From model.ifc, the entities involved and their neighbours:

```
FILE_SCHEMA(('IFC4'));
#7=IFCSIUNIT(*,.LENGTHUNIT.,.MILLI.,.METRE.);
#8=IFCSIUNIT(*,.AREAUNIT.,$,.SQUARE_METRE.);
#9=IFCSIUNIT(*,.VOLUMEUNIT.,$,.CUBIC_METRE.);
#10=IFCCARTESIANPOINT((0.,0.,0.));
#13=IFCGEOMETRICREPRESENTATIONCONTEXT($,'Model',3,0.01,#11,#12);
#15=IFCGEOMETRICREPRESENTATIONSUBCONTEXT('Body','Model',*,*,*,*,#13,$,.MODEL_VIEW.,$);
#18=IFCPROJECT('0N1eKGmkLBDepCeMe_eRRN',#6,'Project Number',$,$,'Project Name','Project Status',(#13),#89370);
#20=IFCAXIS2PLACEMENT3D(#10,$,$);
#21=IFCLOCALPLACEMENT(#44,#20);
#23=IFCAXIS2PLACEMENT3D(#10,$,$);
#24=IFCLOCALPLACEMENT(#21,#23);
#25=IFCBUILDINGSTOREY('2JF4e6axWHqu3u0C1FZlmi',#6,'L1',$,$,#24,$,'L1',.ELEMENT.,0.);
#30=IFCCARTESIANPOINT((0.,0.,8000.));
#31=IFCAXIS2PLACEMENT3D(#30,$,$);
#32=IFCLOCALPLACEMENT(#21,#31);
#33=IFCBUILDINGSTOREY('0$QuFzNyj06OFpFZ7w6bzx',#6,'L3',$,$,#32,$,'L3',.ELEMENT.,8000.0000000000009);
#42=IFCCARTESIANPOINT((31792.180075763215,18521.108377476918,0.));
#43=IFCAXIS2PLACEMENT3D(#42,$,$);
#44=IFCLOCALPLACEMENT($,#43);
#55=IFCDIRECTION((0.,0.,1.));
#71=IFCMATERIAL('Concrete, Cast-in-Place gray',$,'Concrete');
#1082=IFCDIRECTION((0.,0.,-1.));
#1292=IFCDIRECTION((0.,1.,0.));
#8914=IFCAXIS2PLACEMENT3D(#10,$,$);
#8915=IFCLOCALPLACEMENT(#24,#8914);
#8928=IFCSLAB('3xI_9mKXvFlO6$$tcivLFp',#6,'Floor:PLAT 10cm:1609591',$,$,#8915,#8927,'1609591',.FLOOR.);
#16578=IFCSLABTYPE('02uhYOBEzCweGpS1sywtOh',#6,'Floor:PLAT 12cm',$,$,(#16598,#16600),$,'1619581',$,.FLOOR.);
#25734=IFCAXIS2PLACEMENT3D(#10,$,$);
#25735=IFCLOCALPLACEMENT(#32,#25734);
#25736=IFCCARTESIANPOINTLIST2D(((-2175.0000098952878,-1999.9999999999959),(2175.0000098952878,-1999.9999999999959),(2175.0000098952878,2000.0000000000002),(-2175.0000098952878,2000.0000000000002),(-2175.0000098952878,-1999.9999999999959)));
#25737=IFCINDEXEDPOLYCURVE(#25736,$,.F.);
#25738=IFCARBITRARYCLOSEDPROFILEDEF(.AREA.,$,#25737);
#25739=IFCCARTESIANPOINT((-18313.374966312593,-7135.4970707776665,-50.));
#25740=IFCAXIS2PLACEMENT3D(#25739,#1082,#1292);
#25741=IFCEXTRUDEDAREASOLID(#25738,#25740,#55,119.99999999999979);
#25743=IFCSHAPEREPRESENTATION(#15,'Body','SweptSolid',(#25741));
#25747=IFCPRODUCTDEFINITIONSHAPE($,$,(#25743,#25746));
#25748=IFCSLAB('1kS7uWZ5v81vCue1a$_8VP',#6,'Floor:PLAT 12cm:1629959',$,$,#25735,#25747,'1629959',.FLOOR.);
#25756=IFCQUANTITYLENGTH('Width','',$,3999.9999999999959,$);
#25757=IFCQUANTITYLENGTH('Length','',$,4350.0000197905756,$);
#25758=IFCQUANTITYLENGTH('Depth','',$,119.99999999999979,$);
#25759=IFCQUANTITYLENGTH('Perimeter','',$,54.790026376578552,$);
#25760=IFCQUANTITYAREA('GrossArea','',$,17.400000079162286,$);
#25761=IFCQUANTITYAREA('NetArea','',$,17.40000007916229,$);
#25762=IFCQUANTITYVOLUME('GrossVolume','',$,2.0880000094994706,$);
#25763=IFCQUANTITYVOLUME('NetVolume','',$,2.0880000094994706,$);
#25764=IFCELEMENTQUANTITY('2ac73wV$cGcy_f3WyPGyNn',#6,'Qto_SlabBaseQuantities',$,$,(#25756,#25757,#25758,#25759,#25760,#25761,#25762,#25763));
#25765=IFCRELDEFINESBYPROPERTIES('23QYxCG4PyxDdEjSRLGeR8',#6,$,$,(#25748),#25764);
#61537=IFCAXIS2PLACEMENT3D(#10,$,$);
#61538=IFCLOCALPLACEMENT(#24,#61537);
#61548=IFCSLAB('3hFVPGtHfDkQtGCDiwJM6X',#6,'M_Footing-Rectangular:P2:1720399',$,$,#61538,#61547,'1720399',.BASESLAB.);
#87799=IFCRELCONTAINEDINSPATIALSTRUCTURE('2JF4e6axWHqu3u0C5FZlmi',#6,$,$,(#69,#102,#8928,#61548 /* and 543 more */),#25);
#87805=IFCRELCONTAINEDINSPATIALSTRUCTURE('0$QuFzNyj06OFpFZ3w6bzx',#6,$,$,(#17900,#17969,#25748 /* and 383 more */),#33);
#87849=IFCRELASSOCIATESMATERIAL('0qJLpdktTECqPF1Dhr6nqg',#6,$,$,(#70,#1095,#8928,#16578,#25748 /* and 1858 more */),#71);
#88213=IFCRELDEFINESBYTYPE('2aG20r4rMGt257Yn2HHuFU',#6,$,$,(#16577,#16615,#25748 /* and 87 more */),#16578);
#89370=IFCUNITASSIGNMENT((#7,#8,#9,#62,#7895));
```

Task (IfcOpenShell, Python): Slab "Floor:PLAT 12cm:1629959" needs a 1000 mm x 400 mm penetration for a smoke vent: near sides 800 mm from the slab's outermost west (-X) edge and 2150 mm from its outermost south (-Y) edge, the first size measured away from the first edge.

```python
import numpy as np
import ifcopenshell
import ifcopenshell.api.feature
import ifcopenshell.api.geometry
import ifcopenshell.api.pset
import ifcopenshell.api.root
import ifcopenshell.geom
import ifcopenshell.util.element
import ifcopenshell.util.placement
import ifcopenshell.util.representation
import ifcopenshell.util.shape
import ifcopenshell.util.unit

model = ifcopenshell.open("model.ifc")
unit_scale = ifcopenshell.util.unit.calculate_unit_scale(model)
area_scale = ifcopenshell.util.unit.calculate_unit_scale(model, "AREAUNIT")
volume_scale = ifcopenshell.util.unit.calculate_unit_scale(model, "VOLUMEUNIT")
settings = ifcopenshell.geom.settings()


def volume(element):
    """Net volume in cubic metres, openings subtracted."""
    shape = ifcopenshell.geom.create_shape(settings, element)
    return ifcopenshell.util.shape.get_volume(shape.geometry)


slab = model.by_guid("1kS7uWZ5v81vCue1a$_8VP")
before = volume(slab)

# Extent in the slab's own axes, in metres. The edges named are its -X and -Y sides.
slab_shape = ifcopenshell.geom.create_shape(settings, slab)
vertices = ifcopenshell.util.shape.get_vertices(slab_shape.geometry)
x_min, y_min, bottom = vertices.min(axis=0)
top = vertices[:, 2].max()

opening = ifcopenshell.api.root.create_entity(model, ifc_class="IfcOpeningElement", name="Smoke vent opening", predefined_type="OPENING")
context = ifcopenshell.util.representation.get_context(model, "Model", "Body", "MODEL_VIEW")
width, depth = 1, 0.4
outline = [(0.0, 0.0), (width, 0.0), (width, depth), (0.0, depth), (0.0, 0.0)]
# Overshoot both faces by 50 mm so the cut is clean.
shape = ifcopenshell.api.geometry.add_slab_representation(
    model, context=context, depth=top - bottom + 0.1, polyline=outline
)
ifcopenshell.api.geometry.assign_representation(model, product=opening, representation=shape)

matrix = ifcopenshell.util.placement.get_local_placement(slab.ObjectPlacement)
matrix[:, 3] = matrix @ np.append(np.array([x_min + 0.8, y_min + 2.15, bottom - 0.05]) / unit_scale, 1.0)
ifcopenshell.api.geometry.edit_object_placement(model, product=opening, matrix=matrix, is_si=False)
ifcopenshell.api.feature.add_feature(model, feature=opening, element=slab)

after = volume(slab)

# Update the slab's stored quantities.
qto = model.by_id(ifcopenshell.util.element.get_pset(slab, "Qto_SlabBaseQuantities", should_inherit=False)["id"])
ifcopenshell.api.pset.edit_qto(model, qto=qto, properties={
    "NetArea": after / (top - bottom) / area_scale,
    "NetVolume": after / volume_scale,
})

print(f"slab volume {before:.3f} -> {after:.3f} m3")

model.write("model_edited.ifc")
```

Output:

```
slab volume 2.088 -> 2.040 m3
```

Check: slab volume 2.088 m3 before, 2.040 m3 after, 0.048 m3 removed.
